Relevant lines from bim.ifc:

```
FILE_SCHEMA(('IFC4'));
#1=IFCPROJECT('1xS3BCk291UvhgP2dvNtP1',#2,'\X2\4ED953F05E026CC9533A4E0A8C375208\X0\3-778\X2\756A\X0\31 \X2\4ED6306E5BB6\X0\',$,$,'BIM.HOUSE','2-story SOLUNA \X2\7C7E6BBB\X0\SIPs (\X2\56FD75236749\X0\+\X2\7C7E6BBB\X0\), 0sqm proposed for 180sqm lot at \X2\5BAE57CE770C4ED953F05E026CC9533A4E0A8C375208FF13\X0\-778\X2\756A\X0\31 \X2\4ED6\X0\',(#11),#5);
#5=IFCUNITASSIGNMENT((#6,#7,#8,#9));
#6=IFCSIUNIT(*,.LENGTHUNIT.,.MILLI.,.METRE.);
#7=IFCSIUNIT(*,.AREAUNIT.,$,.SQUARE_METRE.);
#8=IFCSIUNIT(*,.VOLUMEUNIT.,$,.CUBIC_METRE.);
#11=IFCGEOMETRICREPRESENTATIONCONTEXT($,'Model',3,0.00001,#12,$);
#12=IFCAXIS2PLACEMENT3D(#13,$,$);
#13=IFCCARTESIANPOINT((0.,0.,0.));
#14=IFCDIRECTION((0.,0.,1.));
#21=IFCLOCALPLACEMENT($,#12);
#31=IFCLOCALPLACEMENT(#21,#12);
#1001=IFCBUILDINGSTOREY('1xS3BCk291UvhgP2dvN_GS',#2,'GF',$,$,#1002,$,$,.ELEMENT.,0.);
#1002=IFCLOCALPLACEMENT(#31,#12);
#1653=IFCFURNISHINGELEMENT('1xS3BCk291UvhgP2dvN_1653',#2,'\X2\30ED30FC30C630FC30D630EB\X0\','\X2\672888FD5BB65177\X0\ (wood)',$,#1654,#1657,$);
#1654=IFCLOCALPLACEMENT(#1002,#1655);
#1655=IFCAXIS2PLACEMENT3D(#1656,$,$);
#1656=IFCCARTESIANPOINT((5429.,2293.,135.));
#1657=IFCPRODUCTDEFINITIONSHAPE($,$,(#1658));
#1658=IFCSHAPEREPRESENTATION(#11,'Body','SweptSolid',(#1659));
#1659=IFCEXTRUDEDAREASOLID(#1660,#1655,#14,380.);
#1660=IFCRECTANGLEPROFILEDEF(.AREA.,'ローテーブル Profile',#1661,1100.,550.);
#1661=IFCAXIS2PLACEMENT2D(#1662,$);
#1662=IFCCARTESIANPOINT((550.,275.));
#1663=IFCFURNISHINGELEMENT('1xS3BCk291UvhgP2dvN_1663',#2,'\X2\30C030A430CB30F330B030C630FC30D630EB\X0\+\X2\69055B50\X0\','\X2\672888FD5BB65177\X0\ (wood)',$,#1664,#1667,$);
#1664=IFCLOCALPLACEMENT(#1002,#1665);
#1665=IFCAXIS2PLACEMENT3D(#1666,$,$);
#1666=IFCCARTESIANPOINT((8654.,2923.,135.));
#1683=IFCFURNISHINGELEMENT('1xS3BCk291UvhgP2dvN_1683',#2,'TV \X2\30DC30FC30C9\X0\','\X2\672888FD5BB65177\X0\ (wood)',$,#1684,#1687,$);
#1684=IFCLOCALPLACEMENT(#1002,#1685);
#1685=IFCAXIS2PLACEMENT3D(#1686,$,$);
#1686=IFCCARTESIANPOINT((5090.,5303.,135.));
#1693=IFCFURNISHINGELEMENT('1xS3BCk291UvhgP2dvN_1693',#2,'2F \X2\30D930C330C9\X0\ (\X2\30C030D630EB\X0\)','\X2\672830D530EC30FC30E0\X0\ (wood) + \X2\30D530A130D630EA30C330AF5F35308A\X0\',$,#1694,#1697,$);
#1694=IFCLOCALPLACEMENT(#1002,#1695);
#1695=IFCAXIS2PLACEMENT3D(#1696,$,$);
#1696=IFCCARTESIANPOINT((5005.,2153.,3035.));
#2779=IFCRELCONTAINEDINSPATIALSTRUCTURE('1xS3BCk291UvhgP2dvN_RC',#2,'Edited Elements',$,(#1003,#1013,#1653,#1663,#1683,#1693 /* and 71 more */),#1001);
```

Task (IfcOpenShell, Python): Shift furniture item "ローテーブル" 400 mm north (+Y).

```python
import ifcopenshell
import ifcopenshell.api.geometry
import ifcopenshell.util.placement
import ifcopenshell.util.unit

model = ifcopenshell.open("bim.ifc")
unit_scale = ifcopenshell.util.unit.calculate_unit_scale(model)

item = model.by_guid("1xS3BCk291UvhgP2dvN_1653")
matrix = ifcopenshell.util.placement.get_local_placement(item.ObjectPlacement)
matrix[1, 3] += 0.4 / unit_scale
ifcopenshell.api.geometry.edit_object_placement(model, product=item, matrix=matrix, is_si=False)

print(ifcopenshell.util.placement.get_local_placement(item.ObjectPlacement).round(3) + 0.0)

model.write("bim-out.ifc")
```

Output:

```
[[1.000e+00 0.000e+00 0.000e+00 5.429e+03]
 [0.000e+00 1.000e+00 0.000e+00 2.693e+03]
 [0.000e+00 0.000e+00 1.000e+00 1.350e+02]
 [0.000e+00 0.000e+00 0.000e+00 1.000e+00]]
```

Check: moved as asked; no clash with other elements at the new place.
